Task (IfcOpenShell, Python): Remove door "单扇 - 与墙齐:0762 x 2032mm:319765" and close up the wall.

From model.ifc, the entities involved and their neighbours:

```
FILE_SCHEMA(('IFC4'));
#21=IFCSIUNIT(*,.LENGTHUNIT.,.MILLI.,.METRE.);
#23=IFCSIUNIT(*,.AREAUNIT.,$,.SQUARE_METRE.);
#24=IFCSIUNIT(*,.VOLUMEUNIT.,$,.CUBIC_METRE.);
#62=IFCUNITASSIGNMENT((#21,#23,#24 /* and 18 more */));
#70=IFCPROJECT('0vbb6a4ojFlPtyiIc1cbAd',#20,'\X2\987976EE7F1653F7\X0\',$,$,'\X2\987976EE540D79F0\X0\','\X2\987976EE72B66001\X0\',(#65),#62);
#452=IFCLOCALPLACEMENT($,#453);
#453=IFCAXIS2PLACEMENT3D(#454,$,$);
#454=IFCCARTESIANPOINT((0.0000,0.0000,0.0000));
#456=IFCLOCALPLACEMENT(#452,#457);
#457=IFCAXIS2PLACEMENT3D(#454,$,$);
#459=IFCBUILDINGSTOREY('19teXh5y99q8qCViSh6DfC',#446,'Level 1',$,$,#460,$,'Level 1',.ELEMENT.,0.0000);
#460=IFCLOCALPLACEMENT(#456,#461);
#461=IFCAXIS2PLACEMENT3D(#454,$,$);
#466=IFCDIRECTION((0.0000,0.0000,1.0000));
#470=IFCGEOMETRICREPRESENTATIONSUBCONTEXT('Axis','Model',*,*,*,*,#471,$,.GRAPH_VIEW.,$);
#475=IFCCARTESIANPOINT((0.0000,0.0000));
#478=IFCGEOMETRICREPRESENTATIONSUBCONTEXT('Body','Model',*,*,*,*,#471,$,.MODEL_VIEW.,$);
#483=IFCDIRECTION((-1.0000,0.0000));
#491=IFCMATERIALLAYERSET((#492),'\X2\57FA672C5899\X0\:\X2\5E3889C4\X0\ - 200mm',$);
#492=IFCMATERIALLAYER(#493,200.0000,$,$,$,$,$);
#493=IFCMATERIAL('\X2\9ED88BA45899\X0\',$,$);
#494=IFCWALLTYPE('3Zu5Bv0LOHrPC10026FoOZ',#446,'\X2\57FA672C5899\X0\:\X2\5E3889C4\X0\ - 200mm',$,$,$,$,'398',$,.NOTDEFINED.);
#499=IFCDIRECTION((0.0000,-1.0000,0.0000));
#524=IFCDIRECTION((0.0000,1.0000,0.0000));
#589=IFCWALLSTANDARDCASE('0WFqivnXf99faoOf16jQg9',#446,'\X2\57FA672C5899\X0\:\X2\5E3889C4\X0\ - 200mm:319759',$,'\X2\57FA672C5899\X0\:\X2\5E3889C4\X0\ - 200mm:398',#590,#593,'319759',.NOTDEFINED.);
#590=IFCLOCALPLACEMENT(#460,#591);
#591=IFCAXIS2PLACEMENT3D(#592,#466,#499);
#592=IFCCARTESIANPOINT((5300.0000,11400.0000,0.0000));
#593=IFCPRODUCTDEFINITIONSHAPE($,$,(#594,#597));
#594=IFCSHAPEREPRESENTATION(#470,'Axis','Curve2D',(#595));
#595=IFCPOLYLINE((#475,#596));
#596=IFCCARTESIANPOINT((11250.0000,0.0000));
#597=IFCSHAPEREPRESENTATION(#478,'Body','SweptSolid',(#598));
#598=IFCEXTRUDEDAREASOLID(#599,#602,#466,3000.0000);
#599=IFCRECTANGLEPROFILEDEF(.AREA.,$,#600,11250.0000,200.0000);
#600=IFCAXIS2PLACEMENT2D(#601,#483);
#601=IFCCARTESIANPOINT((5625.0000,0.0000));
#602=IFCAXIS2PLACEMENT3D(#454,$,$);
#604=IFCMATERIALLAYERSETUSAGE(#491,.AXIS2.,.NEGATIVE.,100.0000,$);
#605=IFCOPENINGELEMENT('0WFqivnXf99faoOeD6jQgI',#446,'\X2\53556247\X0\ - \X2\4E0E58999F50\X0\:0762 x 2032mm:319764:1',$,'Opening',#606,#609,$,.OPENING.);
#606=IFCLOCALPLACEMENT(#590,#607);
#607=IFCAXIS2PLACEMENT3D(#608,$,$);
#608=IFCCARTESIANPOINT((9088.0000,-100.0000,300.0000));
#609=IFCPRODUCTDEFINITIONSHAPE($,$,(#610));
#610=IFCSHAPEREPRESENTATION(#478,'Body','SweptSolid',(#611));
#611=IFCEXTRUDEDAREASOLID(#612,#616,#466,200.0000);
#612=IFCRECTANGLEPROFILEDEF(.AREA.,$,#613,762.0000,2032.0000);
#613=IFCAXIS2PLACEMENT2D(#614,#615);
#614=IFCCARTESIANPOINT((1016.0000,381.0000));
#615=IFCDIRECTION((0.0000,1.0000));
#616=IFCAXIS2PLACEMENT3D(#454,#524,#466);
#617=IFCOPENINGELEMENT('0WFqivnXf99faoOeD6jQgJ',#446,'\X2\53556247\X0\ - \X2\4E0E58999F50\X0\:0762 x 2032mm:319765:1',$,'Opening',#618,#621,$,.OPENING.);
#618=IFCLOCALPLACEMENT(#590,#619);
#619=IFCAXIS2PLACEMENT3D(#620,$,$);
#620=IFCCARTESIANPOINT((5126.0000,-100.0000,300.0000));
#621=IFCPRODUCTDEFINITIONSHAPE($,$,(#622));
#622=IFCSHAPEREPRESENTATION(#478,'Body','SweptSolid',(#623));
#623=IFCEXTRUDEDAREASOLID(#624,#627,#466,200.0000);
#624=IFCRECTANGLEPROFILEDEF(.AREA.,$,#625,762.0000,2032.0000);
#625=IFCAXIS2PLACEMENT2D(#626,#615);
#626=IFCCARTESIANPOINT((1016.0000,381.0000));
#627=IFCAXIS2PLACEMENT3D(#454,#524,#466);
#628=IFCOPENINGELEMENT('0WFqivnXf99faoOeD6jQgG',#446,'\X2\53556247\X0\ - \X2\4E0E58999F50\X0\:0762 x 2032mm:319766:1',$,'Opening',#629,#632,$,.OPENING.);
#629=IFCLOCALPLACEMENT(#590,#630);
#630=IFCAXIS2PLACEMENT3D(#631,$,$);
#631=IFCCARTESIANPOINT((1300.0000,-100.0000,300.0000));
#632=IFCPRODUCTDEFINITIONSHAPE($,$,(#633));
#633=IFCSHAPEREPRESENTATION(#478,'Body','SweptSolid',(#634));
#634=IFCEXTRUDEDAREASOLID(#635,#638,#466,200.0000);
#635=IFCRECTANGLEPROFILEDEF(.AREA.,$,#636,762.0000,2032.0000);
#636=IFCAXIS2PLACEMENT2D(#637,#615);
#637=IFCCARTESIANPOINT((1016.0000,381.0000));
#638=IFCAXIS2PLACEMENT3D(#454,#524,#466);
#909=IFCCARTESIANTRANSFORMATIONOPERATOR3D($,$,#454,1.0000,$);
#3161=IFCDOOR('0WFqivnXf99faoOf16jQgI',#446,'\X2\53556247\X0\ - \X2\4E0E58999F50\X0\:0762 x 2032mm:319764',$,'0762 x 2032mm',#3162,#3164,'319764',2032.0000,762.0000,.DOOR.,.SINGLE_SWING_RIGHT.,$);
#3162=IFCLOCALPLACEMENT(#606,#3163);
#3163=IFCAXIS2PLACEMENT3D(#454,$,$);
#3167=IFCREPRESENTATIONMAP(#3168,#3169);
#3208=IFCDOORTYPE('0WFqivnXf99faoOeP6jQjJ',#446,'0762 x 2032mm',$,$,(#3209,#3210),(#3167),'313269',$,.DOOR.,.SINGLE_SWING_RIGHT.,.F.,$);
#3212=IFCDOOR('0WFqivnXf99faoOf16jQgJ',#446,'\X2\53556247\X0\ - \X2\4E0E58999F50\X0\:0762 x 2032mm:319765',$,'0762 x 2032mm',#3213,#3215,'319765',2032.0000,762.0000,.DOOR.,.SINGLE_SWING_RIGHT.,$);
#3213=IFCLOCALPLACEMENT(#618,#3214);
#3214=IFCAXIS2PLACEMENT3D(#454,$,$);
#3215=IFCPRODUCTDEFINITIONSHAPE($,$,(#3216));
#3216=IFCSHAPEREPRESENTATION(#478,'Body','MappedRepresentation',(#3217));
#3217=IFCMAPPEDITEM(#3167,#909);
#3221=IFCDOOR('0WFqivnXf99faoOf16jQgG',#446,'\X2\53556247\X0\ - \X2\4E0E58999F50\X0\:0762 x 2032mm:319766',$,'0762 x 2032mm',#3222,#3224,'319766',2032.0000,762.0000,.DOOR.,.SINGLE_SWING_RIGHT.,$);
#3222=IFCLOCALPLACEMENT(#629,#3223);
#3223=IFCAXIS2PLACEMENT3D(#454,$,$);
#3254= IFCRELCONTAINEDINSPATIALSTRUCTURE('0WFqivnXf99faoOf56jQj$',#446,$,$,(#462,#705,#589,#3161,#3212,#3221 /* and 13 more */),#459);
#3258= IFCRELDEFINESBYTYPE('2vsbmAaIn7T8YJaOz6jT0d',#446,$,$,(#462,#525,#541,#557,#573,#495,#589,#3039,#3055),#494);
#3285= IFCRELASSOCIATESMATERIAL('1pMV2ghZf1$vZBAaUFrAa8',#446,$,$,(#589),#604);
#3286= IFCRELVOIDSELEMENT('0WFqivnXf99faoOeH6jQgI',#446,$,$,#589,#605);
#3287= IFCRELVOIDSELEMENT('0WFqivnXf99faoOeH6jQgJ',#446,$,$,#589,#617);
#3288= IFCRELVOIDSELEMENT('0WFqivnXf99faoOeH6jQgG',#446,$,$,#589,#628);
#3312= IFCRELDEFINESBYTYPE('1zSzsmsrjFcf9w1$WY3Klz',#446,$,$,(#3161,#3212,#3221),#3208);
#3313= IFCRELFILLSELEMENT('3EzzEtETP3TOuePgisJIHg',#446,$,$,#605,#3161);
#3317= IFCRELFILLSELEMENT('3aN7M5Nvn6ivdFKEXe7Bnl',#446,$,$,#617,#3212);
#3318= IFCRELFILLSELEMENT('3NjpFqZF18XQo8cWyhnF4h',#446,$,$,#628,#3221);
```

```python
import ifcopenshell
import ifcopenshell.api.feature
import ifcopenshell.api.root
import ifcopenshell.geom
import ifcopenshell.util.shape

model = ifcopenshell.open("model.ifc")
settings = ifcopenshell.geom.settings()


def volume(element):
    """Net volume in cubic metres, openings subtracted."""
    shape = ifcopenshell.geom.create_shape(settings, element)
    return ifcopenshell.util.shape.get_volume(shape.geometry)


door = model.by_guid("0WFqivnXf99faoOf16jQgJ")
opening = door.FillsVoids[0].RelatingOpeningElement
wall = opening.VoidsElements[0].RelatingBuildingElement
before = volume(wall)

ifcopenshell.api.root.remove_product(model, product=door)
ifcopenshell.api.feature.remove_feature(model, feature=opening)

after = volume(wall)

print(f"wall volume {before:.3f} -> {after:.3f} m3")

model.write("model-out.ifc")
```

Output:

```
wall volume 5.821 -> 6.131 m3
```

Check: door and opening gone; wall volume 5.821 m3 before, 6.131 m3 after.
